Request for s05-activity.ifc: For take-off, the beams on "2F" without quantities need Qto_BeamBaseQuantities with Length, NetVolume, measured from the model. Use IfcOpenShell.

First a look at what the model holds.

```python
import ifcopenshell
import ifcopenshell.util.element
import ifcopenshell.util.unit

model = ifcopenshell.open("s05-activity.ifc")
print(model.schema)
for unit_type in ("LENGTHUNIT", "AREAUNIT", "VOLUMEUNIT"):
    print(unit_type, ifcopenshell.util.unit.calculate_unit_scale(model, unit_type))
storey = next(s for s in model.by_type("IfcBuildingStorey") if s.Name == "2F")
beams = [e for e in ifcopenshell.util.element.get_decomposition(storey) if e.is_a("IfcBeam")]
for e in sorted(beams, key=lambda e: e.id()):
    print(e.id(), e.is_a(), e.Name, list(ifcopenshell.util.element.get_psets(e, qtos_only=True)), sep=" | ")
```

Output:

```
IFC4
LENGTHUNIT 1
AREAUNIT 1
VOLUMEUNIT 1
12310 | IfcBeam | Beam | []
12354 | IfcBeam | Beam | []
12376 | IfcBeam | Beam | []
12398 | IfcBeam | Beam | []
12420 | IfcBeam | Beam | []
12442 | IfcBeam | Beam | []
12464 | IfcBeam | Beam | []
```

```python
import ifcopenshell
import ifcopenshell.api.pset
import ifcopenshell.geom
import ifcopenshell.util.element
import ifcopenshell.util.shape
import ifcopenshell.util.unit

model = ifcopenshell.open("s05-activity.ifc")
unit_scale = ifcopenshell.util.unit.calculate_unit_scale(model)
volume_scale = ifcopenshell.util.unit.calculate_unit_scale(model, "VOLUMEUNIT")
settings = ifcopenshell.geom.settings()

storey = next(s for s in model.by_type("IfcBuildingStorey") if s.Name == "2F")
beams = [e for e in ifcopenshell.util.element.get_decomposition(storey) if e.is_a("IfcBeam")]

for e in sorted(beams, key=lambda e: e.id()):
    if ifcopenshell.util.element.get_psets(e, qtos_only=True, should_inherit=False):
        continue
    # Geometry comes back in metres, in the element's own axes.
    shape = ifcopenshell.geom.create_shape(settings, e)
    values = {
        "Length": ifcopenshell.util.shape.get_max_xyz(shape.geometry) / unit_scale,
        "NetVolume": ifcopenshell.util.shape.get_volume(shape.geometry) / volume_scale,
    }
    qto = ifcopenshell.api.pset.add_qto(model, product=e, name="Qto_BeamBaseQuantities")
    ifcopenshell.api.pset.edit_qto(model, qto=qto, properties=values)
    print(e.id(), {k: round(v, 3) for k, v in values.items()})

model.write("s05-activity_updated.ifc")
```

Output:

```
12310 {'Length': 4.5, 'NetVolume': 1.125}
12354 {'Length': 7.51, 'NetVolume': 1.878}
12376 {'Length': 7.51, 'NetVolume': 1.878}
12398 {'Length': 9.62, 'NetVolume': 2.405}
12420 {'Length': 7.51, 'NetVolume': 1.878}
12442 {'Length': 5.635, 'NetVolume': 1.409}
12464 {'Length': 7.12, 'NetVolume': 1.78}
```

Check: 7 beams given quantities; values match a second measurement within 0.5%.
